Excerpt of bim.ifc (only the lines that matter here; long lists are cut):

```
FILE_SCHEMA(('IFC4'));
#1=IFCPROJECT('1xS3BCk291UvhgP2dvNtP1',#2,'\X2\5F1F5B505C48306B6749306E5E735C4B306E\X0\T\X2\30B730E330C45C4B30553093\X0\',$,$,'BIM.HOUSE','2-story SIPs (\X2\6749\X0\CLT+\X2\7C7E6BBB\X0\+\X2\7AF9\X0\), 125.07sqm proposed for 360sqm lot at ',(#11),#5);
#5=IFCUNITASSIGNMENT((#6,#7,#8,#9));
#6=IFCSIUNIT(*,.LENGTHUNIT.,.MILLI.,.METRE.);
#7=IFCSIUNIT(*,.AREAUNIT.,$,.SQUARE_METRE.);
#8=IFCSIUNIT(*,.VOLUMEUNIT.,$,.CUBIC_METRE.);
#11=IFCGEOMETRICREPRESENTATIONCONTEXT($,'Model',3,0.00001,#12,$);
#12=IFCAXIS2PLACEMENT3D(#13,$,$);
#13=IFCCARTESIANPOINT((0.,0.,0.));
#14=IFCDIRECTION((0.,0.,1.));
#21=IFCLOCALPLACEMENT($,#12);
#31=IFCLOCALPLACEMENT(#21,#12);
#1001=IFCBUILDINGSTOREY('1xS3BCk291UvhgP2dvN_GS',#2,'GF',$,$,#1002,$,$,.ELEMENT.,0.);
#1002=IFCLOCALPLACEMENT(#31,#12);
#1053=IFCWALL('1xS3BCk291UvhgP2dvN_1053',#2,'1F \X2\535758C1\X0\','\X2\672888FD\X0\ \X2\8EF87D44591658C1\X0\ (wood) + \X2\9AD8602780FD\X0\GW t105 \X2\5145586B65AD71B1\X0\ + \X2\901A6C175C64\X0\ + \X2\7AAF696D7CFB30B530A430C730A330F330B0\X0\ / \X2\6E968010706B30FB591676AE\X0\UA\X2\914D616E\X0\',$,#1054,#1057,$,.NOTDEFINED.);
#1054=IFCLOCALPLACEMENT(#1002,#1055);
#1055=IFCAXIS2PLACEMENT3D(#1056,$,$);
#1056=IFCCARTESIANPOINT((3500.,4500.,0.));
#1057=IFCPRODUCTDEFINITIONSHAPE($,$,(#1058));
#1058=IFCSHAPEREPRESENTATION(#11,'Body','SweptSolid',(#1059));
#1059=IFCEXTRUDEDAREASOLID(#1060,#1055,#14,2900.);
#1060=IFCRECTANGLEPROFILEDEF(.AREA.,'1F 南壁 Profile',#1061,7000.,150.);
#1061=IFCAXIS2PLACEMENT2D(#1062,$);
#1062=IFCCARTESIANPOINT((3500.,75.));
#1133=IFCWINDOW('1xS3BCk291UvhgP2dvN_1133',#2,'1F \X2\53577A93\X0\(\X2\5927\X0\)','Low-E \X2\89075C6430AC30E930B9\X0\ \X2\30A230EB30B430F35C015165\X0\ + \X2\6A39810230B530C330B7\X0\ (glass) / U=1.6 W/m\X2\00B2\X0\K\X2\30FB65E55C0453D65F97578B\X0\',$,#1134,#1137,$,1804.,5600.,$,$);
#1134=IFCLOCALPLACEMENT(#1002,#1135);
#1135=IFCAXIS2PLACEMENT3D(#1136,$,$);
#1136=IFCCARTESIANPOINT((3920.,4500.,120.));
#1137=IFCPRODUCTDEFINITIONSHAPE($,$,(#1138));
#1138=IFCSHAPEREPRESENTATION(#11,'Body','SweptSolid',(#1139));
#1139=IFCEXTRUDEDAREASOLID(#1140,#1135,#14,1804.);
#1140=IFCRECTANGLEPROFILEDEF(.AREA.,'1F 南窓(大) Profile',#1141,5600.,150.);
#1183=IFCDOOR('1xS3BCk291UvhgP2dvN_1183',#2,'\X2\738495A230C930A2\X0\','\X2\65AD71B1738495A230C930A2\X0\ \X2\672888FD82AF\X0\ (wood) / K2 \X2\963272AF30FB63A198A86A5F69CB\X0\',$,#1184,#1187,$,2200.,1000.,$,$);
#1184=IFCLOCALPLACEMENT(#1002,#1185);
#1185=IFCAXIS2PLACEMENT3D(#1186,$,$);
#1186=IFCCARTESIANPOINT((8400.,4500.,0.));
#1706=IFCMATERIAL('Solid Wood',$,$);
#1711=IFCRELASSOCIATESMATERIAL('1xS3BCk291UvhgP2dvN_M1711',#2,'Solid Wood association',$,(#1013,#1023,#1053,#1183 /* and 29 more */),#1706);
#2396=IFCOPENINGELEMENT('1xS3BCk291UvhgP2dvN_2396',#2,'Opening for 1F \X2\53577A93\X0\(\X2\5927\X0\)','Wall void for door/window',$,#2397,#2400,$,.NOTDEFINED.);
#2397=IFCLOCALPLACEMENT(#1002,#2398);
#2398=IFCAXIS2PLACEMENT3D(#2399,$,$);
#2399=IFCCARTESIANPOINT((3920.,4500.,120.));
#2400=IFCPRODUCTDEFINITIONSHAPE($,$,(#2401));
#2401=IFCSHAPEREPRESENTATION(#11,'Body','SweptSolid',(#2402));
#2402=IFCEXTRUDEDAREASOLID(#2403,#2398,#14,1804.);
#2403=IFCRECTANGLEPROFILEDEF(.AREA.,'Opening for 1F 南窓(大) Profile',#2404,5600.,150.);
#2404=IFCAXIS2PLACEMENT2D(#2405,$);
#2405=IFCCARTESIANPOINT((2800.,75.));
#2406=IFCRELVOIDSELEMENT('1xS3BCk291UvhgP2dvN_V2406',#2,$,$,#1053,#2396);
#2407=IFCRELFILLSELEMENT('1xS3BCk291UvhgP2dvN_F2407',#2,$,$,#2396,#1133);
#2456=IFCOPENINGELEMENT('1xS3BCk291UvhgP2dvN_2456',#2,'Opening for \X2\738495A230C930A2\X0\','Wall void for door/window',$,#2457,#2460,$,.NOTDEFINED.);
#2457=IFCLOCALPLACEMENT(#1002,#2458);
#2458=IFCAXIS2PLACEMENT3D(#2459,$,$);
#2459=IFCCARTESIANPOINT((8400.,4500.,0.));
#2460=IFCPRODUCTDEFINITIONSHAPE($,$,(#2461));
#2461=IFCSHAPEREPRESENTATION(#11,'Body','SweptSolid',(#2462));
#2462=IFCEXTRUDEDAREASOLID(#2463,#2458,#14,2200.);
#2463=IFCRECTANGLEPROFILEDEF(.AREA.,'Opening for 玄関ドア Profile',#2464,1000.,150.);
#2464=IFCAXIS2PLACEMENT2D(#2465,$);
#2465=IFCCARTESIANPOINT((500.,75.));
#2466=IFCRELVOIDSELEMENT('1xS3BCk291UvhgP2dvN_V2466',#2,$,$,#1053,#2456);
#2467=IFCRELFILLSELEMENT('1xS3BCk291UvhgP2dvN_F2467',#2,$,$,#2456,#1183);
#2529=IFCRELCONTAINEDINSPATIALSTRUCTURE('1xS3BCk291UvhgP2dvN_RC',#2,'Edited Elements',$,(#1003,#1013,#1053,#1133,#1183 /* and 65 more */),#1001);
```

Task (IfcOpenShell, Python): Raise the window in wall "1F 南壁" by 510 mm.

```python
import numpy as np
import ifcopenshell
import ifcopenshell.api.geometry
import ifcopenshell.util.placement
import ifcopenshell.util.unit

model = ifcopenshell.open("bim.ifc")
unit_scale = ifcopenshell.util.unit.calculate_unit_scale(model)

window = model.by_id(1133)
opening = window.FillsVoids[0].RelatingOpeningElement
dz = 0.51 / unit_scale

shift = np.array([0.0, 0.0, dz])
# The window is not placed relative to its opening, so move both.
for product in (opening, window):
    matrix = ifcopenshell.util.placement.get_local_placement(product.ObjectPlacement)
    matrix[:3, 3] += shift
    ifcopenshell.api.geometry.edit_object_placement(model, product=product, matrix=matrix, is_si=False)

print(f"moved by {dz * unit_scale:+.3f} m")

model.write("bim_rev.ifc")
```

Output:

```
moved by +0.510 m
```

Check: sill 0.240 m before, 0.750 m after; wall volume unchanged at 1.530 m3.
